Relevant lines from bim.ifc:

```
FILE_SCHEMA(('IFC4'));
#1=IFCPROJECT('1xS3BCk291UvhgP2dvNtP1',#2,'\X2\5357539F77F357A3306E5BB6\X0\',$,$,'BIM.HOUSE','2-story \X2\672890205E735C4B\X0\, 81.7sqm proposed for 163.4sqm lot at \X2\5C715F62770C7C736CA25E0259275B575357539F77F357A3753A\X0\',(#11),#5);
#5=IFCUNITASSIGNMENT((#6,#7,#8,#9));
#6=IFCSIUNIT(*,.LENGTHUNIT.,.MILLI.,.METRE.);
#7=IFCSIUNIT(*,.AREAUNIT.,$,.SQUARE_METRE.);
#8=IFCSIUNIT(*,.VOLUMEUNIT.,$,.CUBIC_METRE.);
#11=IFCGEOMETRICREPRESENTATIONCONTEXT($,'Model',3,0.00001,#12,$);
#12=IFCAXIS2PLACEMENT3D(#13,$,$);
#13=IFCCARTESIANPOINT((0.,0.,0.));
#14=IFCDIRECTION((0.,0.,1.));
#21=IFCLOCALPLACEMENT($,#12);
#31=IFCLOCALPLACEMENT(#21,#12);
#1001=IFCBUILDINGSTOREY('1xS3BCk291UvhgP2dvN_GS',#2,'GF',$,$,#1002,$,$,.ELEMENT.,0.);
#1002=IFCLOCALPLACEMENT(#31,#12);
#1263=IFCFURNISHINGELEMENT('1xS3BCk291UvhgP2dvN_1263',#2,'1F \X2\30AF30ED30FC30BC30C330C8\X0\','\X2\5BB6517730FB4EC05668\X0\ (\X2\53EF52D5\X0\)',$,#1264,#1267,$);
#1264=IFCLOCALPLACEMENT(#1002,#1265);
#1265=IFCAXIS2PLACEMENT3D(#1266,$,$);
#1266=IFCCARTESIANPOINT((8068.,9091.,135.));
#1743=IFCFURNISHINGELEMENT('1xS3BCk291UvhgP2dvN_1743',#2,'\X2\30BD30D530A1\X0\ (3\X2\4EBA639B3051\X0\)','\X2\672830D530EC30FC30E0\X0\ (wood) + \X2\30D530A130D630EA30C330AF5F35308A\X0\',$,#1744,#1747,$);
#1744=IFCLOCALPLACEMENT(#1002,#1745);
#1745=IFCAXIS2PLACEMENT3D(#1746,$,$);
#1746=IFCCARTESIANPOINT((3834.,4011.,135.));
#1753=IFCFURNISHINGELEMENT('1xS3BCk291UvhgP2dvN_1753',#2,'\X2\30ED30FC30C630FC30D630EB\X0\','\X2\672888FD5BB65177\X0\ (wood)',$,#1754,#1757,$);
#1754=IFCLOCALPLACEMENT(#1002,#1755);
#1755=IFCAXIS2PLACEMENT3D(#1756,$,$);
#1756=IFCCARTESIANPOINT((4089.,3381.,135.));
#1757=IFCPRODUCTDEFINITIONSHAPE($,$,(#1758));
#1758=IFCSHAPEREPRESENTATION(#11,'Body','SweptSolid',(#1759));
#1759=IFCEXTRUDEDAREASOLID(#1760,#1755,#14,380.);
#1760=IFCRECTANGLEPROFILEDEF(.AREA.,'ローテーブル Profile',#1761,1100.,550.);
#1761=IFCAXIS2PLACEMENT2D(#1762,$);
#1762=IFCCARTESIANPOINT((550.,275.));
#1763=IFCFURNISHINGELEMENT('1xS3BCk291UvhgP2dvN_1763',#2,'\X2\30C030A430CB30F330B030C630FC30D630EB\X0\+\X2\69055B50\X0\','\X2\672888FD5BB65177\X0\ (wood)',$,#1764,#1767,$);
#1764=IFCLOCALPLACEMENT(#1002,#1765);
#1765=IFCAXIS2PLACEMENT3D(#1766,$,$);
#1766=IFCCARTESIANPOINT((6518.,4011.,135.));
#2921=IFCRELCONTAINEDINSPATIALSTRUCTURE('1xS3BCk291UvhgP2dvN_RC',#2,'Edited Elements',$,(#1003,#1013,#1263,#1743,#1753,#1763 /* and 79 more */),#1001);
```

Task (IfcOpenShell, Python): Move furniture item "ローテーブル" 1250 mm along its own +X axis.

```python
import ifcopenshell
import ifcopenshell.api.geometry
import ifcopenshell.util.placement
import ifcopenshell.util.unit

model = ifcopenshell.open("bim.ifc")
unit_scale = ifcopenshell.util.unit.calculate_unit_scale(model)

item = model.by_guid("1xS3BCk291UvhgP2dvN_1753")
matrix = ifcopenshell.util.placement.get_local_placement(item.ObjectPlacement)
matrix[:3, 3] += matrix[:3, 0] * 1.25 / unit_scale
ifcopenshell.api.geometry.edit_object_placement(model, product=item, matrix=matrix, is_si=False)

print(ifcopenshell.util.placement.get_local_placement(item.ObjectPlacement).round(3) + 0.0)

model.write("bim_rev.ifc")
```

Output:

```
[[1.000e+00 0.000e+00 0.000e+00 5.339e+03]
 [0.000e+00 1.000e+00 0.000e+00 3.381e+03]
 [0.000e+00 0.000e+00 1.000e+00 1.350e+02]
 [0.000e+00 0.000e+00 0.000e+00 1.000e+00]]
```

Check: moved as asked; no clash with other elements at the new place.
